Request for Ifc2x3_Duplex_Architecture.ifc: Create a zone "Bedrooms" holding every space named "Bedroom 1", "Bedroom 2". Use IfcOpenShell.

First a look at what the model holds.

```python
import ifcopenshell

model = ifcopenshell.open("Ifc2x3_Duplex_Architecture.ifc")
print(model.schema)
seen = {}
for space in model.by_type("IfcSpace"):
    seen[space.LongName] = seen.get(space.LongName, 0) + 1
for name, count in sorted(seen.items(), key=str):
    print(count, "x", name)
print("zones:", [z.Name for z in model.by_type("IfcZone")][:20])
```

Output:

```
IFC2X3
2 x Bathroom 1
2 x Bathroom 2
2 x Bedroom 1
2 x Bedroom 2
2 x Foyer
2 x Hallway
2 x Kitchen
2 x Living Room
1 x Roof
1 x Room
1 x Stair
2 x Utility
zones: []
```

```python
import ifcopenshell
import ifcopenshell.api.group
import ifcopenshell.api.root

model = ifcopenshell.open("Ifc2x3_Duplex_Architecture.ifc")

names = {"Bedroom 1", "Bedroom 2"}
spaces = [s for s in model.by_type("IfcSpace") if s.LongName in names]

zone = ifcopenshell.api.root.create_entity(model, ifc_class="IfcZone", name="Bedrooms")
ifcopenshell.api.group.assign_group(model, products=spaces, group=zone)
print(len(spaces), "spaces in", zone.Name)

model.write("Ifc2x3_Duplex_Architecture_rev.ifc")
```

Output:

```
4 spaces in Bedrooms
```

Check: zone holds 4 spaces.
